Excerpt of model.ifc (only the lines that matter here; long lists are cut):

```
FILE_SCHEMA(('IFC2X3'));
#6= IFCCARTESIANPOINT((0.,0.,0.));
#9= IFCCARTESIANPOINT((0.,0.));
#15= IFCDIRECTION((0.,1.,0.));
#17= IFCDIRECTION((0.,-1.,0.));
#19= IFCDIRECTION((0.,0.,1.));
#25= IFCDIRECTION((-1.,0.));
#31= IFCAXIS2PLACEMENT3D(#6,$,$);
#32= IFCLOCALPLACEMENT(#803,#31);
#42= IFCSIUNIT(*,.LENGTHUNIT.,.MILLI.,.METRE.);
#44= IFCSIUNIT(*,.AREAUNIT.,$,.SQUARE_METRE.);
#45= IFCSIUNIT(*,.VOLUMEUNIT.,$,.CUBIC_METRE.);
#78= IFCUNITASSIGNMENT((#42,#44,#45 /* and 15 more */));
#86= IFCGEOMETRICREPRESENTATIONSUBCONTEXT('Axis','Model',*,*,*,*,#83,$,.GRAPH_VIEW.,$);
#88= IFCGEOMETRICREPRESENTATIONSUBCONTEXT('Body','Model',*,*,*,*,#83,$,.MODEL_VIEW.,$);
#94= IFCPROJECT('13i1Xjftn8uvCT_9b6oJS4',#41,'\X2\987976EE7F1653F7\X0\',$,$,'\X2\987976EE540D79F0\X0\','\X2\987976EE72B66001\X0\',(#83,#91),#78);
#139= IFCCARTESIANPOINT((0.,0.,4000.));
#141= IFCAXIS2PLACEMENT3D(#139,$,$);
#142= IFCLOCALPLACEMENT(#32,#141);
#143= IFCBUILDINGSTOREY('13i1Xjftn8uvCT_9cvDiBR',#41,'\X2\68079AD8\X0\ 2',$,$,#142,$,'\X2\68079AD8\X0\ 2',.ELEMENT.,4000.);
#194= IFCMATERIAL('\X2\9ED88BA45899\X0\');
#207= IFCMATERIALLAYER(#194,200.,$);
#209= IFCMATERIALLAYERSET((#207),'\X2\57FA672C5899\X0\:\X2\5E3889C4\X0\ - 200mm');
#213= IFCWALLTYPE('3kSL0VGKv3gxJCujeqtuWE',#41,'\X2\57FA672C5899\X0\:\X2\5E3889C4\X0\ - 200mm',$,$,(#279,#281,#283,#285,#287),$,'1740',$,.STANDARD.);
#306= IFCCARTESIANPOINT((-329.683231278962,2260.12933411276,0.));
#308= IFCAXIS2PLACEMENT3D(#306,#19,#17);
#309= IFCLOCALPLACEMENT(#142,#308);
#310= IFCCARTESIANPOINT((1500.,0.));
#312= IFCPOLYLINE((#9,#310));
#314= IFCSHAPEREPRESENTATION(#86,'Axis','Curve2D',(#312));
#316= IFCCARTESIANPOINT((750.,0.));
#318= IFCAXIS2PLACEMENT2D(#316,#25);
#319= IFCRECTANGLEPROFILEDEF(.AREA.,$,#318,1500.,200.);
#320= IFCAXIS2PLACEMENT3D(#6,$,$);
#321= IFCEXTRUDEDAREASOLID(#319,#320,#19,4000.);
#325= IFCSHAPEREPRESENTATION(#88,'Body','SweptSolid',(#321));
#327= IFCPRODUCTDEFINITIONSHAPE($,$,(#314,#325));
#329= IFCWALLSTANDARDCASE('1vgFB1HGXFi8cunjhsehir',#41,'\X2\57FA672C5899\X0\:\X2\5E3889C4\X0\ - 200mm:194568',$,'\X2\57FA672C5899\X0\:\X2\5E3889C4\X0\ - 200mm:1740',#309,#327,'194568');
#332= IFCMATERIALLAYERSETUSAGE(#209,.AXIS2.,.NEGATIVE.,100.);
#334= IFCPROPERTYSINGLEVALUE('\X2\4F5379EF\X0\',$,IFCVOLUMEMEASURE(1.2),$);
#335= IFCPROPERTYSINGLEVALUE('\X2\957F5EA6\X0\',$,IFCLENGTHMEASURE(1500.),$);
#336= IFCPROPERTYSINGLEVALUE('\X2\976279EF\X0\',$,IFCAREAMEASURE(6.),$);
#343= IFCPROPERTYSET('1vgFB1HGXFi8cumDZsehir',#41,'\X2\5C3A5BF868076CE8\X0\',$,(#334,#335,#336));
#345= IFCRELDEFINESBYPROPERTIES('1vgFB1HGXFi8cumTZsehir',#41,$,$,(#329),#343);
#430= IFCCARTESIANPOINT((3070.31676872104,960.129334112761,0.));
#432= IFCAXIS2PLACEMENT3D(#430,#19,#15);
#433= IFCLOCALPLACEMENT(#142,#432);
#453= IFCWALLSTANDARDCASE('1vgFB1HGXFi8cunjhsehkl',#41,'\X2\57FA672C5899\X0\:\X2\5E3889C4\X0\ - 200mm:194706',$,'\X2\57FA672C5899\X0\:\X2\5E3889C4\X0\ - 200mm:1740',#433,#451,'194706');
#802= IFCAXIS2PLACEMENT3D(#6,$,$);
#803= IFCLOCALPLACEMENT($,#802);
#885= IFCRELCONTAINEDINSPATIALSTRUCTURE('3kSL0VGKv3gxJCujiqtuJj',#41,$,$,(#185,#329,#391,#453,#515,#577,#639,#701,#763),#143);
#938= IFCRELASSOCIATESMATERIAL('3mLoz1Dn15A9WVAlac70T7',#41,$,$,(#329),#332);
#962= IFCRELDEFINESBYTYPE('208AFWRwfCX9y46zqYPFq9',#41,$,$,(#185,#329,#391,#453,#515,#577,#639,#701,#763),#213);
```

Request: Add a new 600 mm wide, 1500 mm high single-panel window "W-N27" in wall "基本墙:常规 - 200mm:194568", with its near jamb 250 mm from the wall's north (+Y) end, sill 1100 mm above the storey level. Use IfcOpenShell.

```python
import numpy as np
import ifcopenshell
import ifcopenshell.api.feature
import ifcopenshell.api.geometry
import ifcopenshell.api.pset
import ifcopenshell.api.root
import ifcopenshell.api.spatial
import ifcopenshell.api.type
import ifcopenshell.geom
import ifcopenshell.util.element
import ifcopenshell.util.placement
import ifcopenshell.util.representation
import ifcopenshell.util.shape
import ifcopenshell.util.unit

model = ifcopenshell.open("model.ifc")
unit_scale = ifcopenshell.util.unit.calculate_unit_scale(model)
area_scale = ifcopenshell.util.unit.calculate_unit_scale(model, "AREAUNIT")
volume_scale = ifcopenshell.util.unit.calculate_unit_scale(model, "VOLUMEUNIT")
settings = ifcopenshell.geom.settings()


def volume(element):
    """Net volume in cubic metres, openings subtracted."""
    shape = ifcopenshell.geom.create_shape(settings, element)
    return ifcopenshell.util.shape.get_volume(shape.geometry)


wall = model.by_guid("1vgFB1HGXFi8cunjhsehir")
storey = ifcopenshell.util.element.get_container(wall, ifc_class="IfcBuildingStorey")
context = ifcopenshell.util.representation.get_context(model, "Model", "Body", "MODEL_VIEW")
before = volume(wall)

width, height, from_end, sill = 0.6, 1.5, 0.25, 1.1  # metres

# The wall runs along its own X axis, and the end named is its -X end.
wall_shape = ifcopenshell.geom.create_shape(settings, wall)
x, y, z = ifcopenshell.util.shape.get_vertices(wall_shape.geometry).T
start = x.min() + from_end
face, thickness = float(y.min()), float(y.max() - y.min())
wall_matrix = ifcopenshell.util.placement.get_local_placement(wall.ObjectPlacement)
level = ifcopenshell.util.placement.get_local_placement(storey.ObjectPlacement)[2, 3]


def in_wall(x, y):
    """Placement at x, y metres in the wall's axes, at sill height."""
    matrix = wall_matrix.copy()
    matrix[:, 3] = wall_matrix @ np.array([x / unit_scale, y / unit_scale, 0.0, 1.0])
    matrix[2, 3] = level + sill / unit_scale
    return matrix


# Opening: a box that overshoots both wall faces by 50 mm.
opening = ifcopenshell.api.root.create_entity(model, ifc_class="IfcOpeningElement")
box = ifcopenshell.api.geometry.add_wall_representation(
    model, context=context, length=width, height=height, thickness=thickness + 0.1
)
ifcopenshell.api.geometry.assign_representation(model, product=opening, representation=box)
ifcopenshell.api.geometry.edit_object_placement(model, product=opening, matrix=in_wall(start, face - 0.05), is_si=False)
ifcopenshell.api.feature.add_feature(model, feature=opening, element=wall)

window = ifcopenshell.api.root.create_entity(model, ifc_class="IfcWindow", name="W-N27")
window.OverallWidth, window.OverallHeight = width / unit_scale, height / unit_scale
body = ifcopenshell.api.geometry.add_window_representation(
    model,
    context=context,
    overall_width=window.OverallWidth,
    overall_height=window.OverallHeight,
    partition_type="SINGLE_PANEL",
)
ifcopenshell.api.geometry.assign_representation(model, product=window, representation=body)
ifcopenshell.api.spatial.assign_container(model, products=[window], relating_structure=storey)
fills = ifcopenshell.api.feature.add_filling(model, opening=opening, element=window)
fills.OwnerHistory = window.OwnerHistory  # required in IFC2X3

# IFC2X3 keeps the operation on the window style.
style = ifcopenshell.api.root.create_entity(model, ifc_class="IfcWindowStyle", name="W-N27")
style.OperationType, style.ConstructionType = "SINGLE_PANEL", "NOTDEFINED"
style.ParameterTakesPrecedence = style.Sizeable = False
ifcopenshell.api.type.assign_type(model, related_objects=[window], relating_type=style)

# Centre the window in the wall's thickness.
ifcopenshell.api.geometry.edit_object_placement(model, product=window, matrix=in_wall(start, face), is_si=False)
window_shape = ifcopenshell.geom.create_shape(settings, window)
depth = ifcopenshell.util.shape.get_vertices(window_shape.geometry)[:, 1]
offset = face + thickness / 2 - (depth.min() + depth.max()) / 2
ifcopenshell.api.geometry.edit_object_placement(model, product=window, matrix=in_wall(start, offset), is_si=False)

after = volume(wall)

# Update the wall's stored quantities.
pset = model.by_id(ifcopenshell.util.element.get_pset(wall, "尺寸标注", should_inherit=False)["id"])
ifcopenshell.api.pset.edit_pset(model, pset=pset, properties={
    "体积": model.create_entity("IfcVolumeMeasure", after / volume_scale),
    "面积": model.create_entity("IfcAreaMeasure", after / thickness / area_scale),
})

print(f"wall volume {before:.3f} -> {after:.3f} m3")

model.write("model_rev.ifc")
```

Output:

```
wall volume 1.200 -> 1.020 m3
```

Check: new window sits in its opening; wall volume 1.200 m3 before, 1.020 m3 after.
